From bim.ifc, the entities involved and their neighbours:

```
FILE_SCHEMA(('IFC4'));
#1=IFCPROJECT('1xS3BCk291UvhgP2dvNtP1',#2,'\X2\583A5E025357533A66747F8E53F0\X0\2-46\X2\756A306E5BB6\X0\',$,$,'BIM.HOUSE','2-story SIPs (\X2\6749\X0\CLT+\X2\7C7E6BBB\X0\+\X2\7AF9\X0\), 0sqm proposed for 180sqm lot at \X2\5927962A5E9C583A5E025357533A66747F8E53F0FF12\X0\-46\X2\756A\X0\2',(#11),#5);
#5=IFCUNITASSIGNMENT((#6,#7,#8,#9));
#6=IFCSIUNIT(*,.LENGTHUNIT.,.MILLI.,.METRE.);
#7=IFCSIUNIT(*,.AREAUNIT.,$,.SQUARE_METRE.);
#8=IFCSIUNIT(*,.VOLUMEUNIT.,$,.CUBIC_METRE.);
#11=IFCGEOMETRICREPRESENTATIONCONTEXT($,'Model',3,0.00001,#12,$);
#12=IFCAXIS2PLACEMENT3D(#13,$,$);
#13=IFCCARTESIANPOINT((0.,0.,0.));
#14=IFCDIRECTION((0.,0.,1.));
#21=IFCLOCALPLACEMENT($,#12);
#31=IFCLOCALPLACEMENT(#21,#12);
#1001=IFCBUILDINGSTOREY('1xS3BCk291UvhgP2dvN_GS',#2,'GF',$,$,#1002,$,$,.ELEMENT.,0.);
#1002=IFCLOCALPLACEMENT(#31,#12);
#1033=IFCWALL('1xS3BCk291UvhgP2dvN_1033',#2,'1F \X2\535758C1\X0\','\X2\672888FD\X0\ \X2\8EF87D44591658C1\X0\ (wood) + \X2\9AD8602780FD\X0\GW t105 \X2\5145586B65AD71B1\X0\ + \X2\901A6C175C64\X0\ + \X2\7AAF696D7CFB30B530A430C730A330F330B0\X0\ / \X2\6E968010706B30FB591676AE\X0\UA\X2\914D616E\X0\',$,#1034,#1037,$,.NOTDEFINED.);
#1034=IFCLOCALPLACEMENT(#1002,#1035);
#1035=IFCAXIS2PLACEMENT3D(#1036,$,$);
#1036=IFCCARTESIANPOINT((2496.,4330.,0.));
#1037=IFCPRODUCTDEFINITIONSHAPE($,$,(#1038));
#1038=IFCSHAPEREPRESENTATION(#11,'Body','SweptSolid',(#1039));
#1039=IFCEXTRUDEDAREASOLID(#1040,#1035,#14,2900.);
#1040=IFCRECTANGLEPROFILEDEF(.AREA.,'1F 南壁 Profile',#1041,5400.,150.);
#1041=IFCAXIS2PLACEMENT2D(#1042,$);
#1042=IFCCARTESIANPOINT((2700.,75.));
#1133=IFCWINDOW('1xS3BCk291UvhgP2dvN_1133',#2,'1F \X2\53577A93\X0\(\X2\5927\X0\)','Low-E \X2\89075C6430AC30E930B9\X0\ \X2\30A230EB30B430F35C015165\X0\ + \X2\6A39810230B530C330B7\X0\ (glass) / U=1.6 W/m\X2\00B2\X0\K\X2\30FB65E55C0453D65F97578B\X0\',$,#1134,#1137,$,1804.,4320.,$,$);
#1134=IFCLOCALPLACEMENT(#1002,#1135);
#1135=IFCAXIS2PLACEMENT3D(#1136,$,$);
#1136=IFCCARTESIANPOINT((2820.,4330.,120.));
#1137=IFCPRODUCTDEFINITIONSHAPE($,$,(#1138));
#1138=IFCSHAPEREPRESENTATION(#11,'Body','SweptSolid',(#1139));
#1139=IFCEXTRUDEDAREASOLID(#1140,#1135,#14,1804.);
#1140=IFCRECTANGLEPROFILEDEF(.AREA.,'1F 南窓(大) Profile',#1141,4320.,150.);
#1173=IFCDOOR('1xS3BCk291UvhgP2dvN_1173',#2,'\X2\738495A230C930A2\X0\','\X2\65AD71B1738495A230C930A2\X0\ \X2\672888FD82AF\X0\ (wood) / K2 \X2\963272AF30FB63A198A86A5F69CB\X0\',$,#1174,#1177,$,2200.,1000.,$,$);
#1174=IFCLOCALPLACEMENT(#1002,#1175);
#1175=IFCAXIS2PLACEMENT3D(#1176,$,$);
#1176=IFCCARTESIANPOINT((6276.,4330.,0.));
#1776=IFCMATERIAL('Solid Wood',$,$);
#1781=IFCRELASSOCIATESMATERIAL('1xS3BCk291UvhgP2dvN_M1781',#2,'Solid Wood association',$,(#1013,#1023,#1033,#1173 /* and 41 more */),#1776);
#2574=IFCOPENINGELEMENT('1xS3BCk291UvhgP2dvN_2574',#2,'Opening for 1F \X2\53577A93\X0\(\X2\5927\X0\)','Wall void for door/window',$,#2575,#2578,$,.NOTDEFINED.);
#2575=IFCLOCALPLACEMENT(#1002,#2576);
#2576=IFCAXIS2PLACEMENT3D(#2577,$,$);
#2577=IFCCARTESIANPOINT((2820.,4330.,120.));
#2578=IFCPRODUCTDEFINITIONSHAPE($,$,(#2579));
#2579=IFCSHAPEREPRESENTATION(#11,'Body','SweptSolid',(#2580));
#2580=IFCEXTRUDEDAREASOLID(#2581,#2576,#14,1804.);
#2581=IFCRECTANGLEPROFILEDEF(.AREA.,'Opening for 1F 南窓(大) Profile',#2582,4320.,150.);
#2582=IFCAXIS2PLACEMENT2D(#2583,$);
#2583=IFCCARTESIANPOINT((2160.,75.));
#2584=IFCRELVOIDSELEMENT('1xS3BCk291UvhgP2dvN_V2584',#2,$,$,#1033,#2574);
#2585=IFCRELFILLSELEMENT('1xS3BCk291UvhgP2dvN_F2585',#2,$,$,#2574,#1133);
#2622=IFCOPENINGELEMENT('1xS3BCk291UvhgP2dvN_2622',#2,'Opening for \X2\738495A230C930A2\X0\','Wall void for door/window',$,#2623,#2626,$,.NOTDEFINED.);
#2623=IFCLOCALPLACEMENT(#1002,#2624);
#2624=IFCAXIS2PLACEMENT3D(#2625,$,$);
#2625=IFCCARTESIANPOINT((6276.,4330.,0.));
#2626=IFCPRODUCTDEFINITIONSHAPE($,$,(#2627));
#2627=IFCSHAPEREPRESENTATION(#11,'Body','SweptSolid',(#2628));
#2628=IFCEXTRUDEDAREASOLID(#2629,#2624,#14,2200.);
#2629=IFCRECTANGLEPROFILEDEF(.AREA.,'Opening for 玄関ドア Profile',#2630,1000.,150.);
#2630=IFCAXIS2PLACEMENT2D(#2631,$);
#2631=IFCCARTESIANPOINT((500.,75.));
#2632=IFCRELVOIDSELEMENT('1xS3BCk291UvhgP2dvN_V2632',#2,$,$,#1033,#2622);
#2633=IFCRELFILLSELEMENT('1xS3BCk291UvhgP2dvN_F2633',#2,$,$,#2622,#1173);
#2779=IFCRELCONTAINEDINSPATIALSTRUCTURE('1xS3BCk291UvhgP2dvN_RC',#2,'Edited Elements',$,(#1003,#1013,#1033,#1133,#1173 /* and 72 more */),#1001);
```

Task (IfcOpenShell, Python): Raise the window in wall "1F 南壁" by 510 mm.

```python
import numpy as np
import ifcopenshell
import ifcopenshell.api.geometry
import ifcopenshell.util.placement
import ifcopenshell.util.unit

model = ifcopenshell.open("bim.ifc")
unit_scale = ifcopenshell.util.unit.calculate_unit_scale(model)

window = model.by_id(1133)
opening = window.FillsVoids[0].RelatingOpeningElement
dz = 510.0

shift = np.array([0.0, 0.0, dz])
# The window is not placed relative to its opening, so move both.
for product in (opening, window):
    matrix = ifcopenshell.util.placement.get_local_placement(product.ObjectPlacement)
    matrix[:3, 3] += shift
    ifcopenshell.api.geometry.edit_object_placement(model, product=product, matrix=matrix, is_si=False)

print(f"moved by {dz * unit_scale:+.3f} m")

model.write("bim_edited.ifc")
```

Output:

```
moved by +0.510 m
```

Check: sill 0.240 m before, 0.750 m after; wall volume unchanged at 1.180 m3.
